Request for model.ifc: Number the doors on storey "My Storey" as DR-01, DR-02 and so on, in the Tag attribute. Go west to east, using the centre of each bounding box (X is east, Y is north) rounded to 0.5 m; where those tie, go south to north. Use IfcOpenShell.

First a look at what the model holds.

```python
import ifcopenshell
import ifcopenshell.util.element
import ifcopenshell.util.placement

model = ifcopenshell.open("model.ifc")
print(model.schema)
storey = next(s for s in model.by_type("IfcBuildingStorey") if s.Name == "My Storey")
doors = [e for e in ifcopenshell.util.element.get_decomposition(storey) if e.is_a("IfcDoor")]
for e in sorted(doors, key=lambda e: e.id()):
    origin = ifcopenshell.util.placement.get_local_placement(e.ObjectPlacement)[:3, 3]
    print(e.id(), e.Tag, e.Name, origin.round(2) + 0.0, sep=" | ")
```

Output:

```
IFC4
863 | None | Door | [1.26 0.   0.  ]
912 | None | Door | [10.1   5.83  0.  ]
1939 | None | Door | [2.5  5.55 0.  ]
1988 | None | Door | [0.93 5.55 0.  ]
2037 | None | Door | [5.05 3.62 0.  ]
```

```python
import ifcopenshell
import ifcopenshell.geom
import ifcopenshell.util.element
import ifcopenshell.util.shape

model = ifcopenshell.open("model.ifc")
settings = ifcopenshell.geom.settings()
settings.set("use-world-coords", True)


def centre(element):
    shape = ifcopenshell.geom.create_shape(settings, element)
    return ifcopenshell.util.shape.get_bbox_centroid(shape.geometry)


storey = next(s for s in model.by_type("IfcBuildingStorey") if s.Name == "My Storey")
doors = [e for e in ifcopenshell.util.element.get_decomposition(storey) if e.is_a("IfcDoor")]

# Insertion points can sit at a corner or the storey origin, so sort by the geometry (in metres).
centres = {e: centre(e) for e in doors}
doors.sort(key=lambda e: (round(centres[e][0] / 0.5), centres[e][1]))

for i, e in enumerate(doors, start=1):
    number = f"DR-{i:02d}"
    e.Tag = number
    print(e.id(), number)

model.write("model-out.ifc")
```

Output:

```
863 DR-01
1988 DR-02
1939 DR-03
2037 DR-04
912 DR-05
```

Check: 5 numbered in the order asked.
